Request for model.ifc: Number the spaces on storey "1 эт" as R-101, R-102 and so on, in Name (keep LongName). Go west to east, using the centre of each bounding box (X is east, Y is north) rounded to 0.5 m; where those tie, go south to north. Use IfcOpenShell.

First a look at what the model holds.

```python
import ifcopenshell
import ifcopenshell.util.element
import ifcopenshell.util.placement

model = ifcopenshell.open("model.ifc")
print(model.schema)
storey = next(s for s in model.by_type("IfcBuildingStorey") if s.Name == "1 эт")
spaces = [e for e in ifcopenshell.util.element.get_decomposition(storey) if e.is_a("IfcSpace")]
for e in sorted(spaces, key=lambda e: e.id()):
    origin = ifcopenshell.util.placement.get_local_placement(e.ObjectPlacement)[:3, 3]
    print(e.id(), e.Name, e.LongName, origin.round(2) + 0.0, sep=" | ")
```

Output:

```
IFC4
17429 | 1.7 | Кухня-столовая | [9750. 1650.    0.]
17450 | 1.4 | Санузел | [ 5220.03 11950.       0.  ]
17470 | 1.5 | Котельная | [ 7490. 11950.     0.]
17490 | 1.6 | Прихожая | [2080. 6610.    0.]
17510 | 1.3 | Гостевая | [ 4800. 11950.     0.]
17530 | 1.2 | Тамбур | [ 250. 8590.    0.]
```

```python
import ifcopenshell
import ifcopenshell.geom
import ifcopenshell.util.element
import ifcopenshell.util.shape

model = ifcopenshell.open("model.ifc")
settings = ifcopenshell.geom.settings()
settings.set("use-world-coords", True)


def centre(element):
    shape = ifcopenshell.geom.create_shape(settings, element)
    return ifcopenshell.util.shape.get_bbox_centroid(shape.geometry)


storey = next(s for s in model.by_type("IfcBuildingStorey") if s.Name == "1 эт")
spaces = [e for e in ifcopenshell.util.element.get_decomposition(storey) if e.is_a("IfcSpace")]

# Insertion points can sit at a corner or the storey origin, so sort by the geometry (in metres).
centres = {e: centre(e) for e in spaces}
spaces.sort(key=lambda e: (round(centres[e][0] / 0.5), centres[e][1]))

for i, e in enumerate(spaces, start=1):
    number = f"R-1{i:02d}"
    e.Name = number
    print(e.id(), number)

model.write("model_updated.ifc")
```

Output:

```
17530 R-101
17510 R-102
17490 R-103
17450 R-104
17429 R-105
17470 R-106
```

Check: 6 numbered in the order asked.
